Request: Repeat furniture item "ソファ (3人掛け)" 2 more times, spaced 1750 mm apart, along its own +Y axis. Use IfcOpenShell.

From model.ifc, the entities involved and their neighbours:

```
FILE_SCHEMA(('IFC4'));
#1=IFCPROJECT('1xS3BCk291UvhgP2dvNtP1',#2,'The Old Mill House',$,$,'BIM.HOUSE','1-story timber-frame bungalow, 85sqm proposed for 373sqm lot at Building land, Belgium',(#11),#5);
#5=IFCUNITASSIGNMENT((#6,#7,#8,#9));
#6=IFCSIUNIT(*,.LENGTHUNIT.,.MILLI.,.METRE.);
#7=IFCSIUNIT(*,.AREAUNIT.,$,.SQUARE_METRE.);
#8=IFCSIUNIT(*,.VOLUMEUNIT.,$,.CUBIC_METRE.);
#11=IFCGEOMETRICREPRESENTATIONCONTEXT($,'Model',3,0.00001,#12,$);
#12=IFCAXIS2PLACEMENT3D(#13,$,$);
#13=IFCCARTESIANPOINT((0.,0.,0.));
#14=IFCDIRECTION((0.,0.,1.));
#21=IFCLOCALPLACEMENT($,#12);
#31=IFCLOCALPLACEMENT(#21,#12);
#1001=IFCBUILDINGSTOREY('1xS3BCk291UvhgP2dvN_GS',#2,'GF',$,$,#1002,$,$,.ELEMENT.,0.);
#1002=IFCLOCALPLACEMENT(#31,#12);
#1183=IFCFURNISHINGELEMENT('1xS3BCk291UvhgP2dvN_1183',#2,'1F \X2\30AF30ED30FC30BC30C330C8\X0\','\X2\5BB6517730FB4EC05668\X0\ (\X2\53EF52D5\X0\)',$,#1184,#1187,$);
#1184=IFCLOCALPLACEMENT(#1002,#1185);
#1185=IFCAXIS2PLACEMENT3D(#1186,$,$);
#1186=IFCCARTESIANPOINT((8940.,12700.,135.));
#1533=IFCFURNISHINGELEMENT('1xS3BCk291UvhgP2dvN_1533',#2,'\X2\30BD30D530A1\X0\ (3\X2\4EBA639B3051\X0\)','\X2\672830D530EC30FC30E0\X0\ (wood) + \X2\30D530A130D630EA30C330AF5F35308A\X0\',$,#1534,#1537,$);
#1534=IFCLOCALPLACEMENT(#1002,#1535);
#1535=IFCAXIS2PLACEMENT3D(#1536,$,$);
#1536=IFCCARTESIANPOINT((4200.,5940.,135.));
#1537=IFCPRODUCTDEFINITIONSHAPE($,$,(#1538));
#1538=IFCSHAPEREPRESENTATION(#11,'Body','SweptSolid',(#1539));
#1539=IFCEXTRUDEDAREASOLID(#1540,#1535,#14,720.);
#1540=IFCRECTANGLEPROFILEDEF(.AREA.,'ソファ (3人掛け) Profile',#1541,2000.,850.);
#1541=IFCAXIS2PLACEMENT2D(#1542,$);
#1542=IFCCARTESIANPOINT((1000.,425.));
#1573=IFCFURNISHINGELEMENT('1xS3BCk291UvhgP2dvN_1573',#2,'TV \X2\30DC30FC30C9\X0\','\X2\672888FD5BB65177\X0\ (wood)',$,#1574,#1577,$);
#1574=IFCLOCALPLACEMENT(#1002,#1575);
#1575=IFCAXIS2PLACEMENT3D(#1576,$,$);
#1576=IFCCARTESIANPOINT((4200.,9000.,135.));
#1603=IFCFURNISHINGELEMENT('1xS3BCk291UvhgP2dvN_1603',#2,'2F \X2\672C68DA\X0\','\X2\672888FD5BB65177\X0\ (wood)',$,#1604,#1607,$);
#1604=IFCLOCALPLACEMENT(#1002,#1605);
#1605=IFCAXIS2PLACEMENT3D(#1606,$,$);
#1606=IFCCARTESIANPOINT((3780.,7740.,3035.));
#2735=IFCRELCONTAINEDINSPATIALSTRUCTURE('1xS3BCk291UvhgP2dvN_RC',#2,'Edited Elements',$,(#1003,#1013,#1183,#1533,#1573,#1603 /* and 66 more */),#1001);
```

```python
import ifcopenshell
import ifcopenshell.api.geometry
import ifcopenshell.api.root
import ifcopenshell.util.element
import ifcopenshell.util.placement
import ifcopenshell.util.unit

model = ifcopenshell.open("model.ifc")
unit_scale = ifcopenshell.util.unit.calculate_unit_scale(model)


def reuse_history(source, copy):
    """copy_class also copies each property set's owner history, people and application; keep the originals."""
    for rel in copy.IsDefinedBy:
        if rel.is_a("IfcRelDefinesByProperties") and (history := rel.RelatingPropertyDefinition.OwnerHistory):
            rel.RelatingPropertyDefinition.OwnerHistory = source.OwnerHistory
            ifcopenshell.util.element.remove_deep2(model, history)


source = model.by_guid("1xS3BCk291UvhgP2dvN_1533")
base = ifcopenshell.util.placement.get_local_placement(source.ObjectPlacement)
step = base[:3, 1] * 1.75 / unit_scale

for i in range(1, 3):
    copy = ifcopenshell.api.root.copy_class(model, product=source)
    copy.Representation = ifcopenshell.util.element.copy_deep(
        model, source.Representation, exclude=["IfcGeometricRepresentationContext", "IfcRepresentationMap"]
    )
    reuse_history(source, copy)
    matrix = base.copy()
    matrix[:3, 3] += i * step
    print("added at", matrix[:3, 3].round(3) + 0.0)
    ifcopenshell.api.geometry.edit_object_placement(model, product=copy, matrix=matrix, is_si=False)

model.write("model_v2.ifc")
```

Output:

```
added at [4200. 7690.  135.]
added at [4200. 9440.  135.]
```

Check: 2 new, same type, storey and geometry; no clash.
